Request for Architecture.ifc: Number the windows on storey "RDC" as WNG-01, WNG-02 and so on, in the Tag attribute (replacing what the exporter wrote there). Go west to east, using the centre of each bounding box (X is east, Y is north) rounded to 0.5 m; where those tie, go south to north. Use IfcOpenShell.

First a look at what the model holds.

```python
import ifcopenshell
import ifcopenshell.util.element
import ifcopenshell.util.placement

model = ifcopenshell.open("Architecture.ifc")
print(model.schema)
storey = next(s for s in model.by_type("IfcBuildingStorey") if s.Name == "RDC")
windows = [e for e in ifcopenshell.util.element.get_decomposition(storey) if e.is_a("IfcWindow")]
for e in sorted(windows, key=lambda e: e.id()):
    origin = ifcopenshell.util.placement.get_local_placement(e.ObjectPlacement)[:3, 3]
    print(e.id(), e.Tag, e.Name, origin.round(2) + 0.0, sep=" | ")
```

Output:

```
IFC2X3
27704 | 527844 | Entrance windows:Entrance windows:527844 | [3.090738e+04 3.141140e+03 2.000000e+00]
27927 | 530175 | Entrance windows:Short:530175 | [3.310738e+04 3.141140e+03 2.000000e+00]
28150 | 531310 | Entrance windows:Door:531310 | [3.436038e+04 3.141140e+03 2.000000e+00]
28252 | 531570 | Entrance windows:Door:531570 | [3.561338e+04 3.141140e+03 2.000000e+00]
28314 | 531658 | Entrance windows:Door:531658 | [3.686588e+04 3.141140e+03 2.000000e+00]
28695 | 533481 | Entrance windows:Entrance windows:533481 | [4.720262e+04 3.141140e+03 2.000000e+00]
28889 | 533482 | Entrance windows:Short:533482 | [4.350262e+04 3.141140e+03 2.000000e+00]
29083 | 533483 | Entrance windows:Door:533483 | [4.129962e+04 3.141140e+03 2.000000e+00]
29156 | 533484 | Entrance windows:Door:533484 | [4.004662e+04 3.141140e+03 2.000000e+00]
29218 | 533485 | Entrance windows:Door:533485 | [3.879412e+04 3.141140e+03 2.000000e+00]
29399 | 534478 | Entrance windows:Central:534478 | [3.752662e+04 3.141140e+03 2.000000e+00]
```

```python
import ifcopenshell
import ifcopenshell.geom
import ifcopenshell.util.element
import ifcopenshell.util.shape

model = ifcopenshell.open("Architecture.ifc")
settings = ifcopenshell.geom.settings()
settings.set("use-world-coords", True)


def centre(element):
    shape = ifcopenshell.geom.create_shape(settings, element)
    return ifcopenshell.util.shape.get_bbox_centroid(shape.geometry)


storey = next(s for s in model.by_type("IfcBuildingStorey") if s.Name == "RDC")
windows = [e for e in ifcopenshell.util.element.get_decomposition(storey) if e.is_a("IfcWindow")]

# Insertion points can sit at a corner or the storey origin, so sort by the geometry (in metres).
centres = {e: centre(e) for e in windows}
windows.sort(key=lambda e: (round(centres[e][0] / 0.5), centres[e][1]))

for i, e in enumerate(windows, start=1):
    number = f"WNG-{i:02d}"
    e.Tag = number
    print(e.id(), number)

model.write("Architecture_edited.ifc")
```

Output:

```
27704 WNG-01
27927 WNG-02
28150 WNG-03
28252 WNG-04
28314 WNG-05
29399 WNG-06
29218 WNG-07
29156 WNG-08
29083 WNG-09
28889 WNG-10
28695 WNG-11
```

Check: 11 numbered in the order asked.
